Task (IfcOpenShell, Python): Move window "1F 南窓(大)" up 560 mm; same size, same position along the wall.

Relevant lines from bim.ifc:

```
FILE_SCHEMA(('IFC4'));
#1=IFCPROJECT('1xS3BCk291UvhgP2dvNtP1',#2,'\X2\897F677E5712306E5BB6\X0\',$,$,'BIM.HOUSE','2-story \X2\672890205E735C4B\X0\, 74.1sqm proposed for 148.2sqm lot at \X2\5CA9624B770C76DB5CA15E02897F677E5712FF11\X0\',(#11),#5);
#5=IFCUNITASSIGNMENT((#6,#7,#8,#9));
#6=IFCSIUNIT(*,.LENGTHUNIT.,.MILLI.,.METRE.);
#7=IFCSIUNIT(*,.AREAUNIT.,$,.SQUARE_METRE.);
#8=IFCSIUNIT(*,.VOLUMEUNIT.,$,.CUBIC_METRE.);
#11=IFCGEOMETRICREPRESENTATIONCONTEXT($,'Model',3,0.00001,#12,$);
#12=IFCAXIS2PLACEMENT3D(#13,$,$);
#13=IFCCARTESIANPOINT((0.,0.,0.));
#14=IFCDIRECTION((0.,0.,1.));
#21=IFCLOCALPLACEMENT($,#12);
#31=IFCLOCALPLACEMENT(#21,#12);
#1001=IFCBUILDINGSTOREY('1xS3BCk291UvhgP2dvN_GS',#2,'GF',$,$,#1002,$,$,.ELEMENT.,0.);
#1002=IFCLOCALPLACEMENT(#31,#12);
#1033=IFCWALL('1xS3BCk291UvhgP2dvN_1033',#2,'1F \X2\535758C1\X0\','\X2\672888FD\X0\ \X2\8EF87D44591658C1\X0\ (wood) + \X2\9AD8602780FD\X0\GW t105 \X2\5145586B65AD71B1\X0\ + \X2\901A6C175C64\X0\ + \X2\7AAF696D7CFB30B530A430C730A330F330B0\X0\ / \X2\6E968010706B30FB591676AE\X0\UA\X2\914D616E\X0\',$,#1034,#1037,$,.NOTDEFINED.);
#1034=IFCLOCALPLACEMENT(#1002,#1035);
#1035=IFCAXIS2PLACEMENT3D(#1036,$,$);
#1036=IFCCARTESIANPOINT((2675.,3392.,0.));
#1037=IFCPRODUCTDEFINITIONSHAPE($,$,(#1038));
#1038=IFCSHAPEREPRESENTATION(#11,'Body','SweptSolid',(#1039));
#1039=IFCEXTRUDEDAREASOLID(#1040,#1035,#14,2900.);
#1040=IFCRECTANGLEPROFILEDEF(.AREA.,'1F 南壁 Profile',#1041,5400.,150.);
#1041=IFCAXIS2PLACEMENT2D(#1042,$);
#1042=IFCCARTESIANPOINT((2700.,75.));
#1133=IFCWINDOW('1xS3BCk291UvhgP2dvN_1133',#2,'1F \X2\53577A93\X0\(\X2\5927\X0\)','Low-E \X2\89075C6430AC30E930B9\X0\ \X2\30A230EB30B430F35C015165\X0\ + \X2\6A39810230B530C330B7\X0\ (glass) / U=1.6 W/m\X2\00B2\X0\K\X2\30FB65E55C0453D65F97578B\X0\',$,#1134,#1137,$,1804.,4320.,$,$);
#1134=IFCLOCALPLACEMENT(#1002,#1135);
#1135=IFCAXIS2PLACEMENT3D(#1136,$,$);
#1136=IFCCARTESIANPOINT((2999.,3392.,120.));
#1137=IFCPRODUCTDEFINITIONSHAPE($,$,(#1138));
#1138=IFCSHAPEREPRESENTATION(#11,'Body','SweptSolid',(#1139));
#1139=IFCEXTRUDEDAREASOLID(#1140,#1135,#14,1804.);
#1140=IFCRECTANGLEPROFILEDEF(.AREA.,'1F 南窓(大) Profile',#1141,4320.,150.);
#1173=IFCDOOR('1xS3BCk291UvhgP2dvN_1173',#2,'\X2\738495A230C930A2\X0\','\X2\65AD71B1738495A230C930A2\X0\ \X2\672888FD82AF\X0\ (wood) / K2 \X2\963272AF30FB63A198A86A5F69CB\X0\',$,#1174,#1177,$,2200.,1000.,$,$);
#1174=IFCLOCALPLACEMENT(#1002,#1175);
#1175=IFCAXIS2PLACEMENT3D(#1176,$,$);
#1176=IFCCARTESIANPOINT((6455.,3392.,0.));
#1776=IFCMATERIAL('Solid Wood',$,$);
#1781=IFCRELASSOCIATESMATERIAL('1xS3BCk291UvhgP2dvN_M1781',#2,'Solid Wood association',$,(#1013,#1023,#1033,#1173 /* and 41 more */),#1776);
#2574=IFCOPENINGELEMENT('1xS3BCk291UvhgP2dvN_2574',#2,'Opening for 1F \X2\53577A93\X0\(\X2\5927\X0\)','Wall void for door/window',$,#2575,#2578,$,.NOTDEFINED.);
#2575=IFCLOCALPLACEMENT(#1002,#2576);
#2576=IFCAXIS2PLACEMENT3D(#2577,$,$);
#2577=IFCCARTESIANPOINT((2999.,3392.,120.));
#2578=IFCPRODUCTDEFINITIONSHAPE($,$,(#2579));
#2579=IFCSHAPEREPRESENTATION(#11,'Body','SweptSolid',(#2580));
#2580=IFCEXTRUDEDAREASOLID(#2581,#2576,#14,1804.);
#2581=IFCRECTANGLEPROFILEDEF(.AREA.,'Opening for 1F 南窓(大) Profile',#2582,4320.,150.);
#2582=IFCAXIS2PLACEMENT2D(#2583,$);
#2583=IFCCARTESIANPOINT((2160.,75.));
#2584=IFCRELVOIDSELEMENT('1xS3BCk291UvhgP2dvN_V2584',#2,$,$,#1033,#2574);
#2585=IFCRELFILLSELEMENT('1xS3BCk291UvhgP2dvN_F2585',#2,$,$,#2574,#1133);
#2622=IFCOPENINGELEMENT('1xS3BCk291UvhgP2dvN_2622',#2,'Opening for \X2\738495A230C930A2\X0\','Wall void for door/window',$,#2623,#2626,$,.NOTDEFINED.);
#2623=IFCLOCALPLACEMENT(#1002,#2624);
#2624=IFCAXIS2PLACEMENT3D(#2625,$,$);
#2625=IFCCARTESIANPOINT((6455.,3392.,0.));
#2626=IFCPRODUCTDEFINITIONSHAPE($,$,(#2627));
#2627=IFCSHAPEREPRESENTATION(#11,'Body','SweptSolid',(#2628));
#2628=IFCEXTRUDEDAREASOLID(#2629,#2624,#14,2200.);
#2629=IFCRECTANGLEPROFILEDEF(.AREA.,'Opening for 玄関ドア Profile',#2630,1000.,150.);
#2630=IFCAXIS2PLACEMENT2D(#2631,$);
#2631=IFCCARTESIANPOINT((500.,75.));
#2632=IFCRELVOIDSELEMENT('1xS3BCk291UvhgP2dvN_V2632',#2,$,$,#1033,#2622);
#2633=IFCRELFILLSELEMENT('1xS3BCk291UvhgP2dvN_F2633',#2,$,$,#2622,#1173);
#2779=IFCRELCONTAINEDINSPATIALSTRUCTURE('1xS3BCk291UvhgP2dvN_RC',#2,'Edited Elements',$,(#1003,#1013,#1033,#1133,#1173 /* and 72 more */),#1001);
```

```python
import numpy as np
import ifcopenshell
import ifcopenshell.api.geometry
import ifcopenshell.util.placement
import ifcopenshell.util.unit

model = ifcopenshell.open("bim.ifc")
unit_scale = ifcopenshell.util.unit.calculate_unit_scale(model)

window = model.by_guid("1xS3BCk291UvhgP2dvN_1133")
opening = window.FillsVoids[0].RelatingOpeningElement
dz = 0.56 / unit_scale

shift = np.array([0.0, 0.0, dz])
# The window is not placed relative to its opening, so move both.
for product in (opening, window):
    matrix = ifcopenshell.util.placement.get_local_placement(product.ObjectPlacement)
    matrix[:3, 3] += shift
    ifcopenshell.api.geometry.edit_object_placement(model, product=product, matrix=matrix, is_si=False)

print(f"moved by {dz * unit_scale:+.3f} m")

model.write("bim_updated.ifc")
```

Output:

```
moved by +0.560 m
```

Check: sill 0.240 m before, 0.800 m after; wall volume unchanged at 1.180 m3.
